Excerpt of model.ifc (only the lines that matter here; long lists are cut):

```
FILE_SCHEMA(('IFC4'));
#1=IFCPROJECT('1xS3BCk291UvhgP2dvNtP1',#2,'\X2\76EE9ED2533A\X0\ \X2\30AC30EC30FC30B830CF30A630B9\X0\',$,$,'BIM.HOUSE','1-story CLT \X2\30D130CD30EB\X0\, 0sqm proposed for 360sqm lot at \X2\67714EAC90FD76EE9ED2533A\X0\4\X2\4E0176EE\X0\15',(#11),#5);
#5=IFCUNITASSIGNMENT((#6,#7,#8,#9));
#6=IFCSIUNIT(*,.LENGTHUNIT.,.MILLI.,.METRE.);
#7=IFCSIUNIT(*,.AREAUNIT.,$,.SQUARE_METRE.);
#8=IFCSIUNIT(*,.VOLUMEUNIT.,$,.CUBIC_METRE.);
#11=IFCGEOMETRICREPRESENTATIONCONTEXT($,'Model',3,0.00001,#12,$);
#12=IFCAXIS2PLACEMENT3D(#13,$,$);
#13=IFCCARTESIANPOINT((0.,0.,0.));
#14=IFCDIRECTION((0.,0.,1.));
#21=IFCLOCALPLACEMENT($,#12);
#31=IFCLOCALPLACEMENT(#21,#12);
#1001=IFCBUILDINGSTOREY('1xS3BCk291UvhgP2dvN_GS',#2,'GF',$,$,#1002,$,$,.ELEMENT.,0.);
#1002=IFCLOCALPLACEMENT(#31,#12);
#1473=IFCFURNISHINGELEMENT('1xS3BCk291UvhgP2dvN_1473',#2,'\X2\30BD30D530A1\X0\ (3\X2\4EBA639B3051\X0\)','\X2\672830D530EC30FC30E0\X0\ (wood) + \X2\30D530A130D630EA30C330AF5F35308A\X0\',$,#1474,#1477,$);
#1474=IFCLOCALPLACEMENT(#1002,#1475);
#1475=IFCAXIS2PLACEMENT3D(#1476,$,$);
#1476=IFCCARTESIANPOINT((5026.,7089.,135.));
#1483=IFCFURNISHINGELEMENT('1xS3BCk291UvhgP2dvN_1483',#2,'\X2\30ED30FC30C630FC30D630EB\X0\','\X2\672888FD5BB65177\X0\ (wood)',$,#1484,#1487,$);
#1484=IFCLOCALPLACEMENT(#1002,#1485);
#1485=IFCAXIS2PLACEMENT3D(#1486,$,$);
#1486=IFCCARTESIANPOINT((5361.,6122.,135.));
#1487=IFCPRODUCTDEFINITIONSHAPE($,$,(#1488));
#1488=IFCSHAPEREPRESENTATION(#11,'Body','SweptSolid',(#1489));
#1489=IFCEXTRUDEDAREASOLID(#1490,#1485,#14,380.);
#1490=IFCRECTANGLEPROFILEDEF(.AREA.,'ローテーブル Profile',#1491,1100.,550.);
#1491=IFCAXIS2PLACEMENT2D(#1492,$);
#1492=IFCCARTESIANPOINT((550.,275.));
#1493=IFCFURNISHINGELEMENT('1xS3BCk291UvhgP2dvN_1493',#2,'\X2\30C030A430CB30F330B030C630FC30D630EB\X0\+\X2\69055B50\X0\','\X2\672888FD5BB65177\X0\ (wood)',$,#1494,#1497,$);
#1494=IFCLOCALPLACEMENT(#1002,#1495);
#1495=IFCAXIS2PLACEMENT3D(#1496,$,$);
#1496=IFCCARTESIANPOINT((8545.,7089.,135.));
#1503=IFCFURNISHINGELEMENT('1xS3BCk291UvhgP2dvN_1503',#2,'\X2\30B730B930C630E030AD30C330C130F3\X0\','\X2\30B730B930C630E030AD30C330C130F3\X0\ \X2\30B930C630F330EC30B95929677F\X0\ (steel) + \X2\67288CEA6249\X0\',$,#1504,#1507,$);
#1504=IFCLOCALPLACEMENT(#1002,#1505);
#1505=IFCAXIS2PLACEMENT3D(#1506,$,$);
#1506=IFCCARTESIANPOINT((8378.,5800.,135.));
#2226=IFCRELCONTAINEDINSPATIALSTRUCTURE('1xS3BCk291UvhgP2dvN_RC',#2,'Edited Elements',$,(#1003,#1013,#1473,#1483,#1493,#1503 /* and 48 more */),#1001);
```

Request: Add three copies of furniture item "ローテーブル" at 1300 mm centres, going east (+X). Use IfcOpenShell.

```python
import numpy as np
import ifcopenshell
import ifcopenshell.api.geometry
import ifcopenshell.api.root
import ifcopenshell.util.element
import ifcopenshell.util.placement
import ifcopenshell.util.unit

model = ifcopenshell.open("model.ifc")
unit_scale = ifcopenshell.util.unit.calculate_unit_scale(model)


def reuse_history(source, copy):
    """copy_class also copies each property set's owner history, people and application; keep the originals."""
    for rel in copy.IsDefinedBy:
        if rel.is_a("IfcRelDefinesByProperties") and (history := rel.RelatingPropertyDefinition.OwnerHistory):
            rel.RelatingPropertyDefinition.OwnerHistory = source.OwnerHistory
            ifcopenshell.util.element.remove_deep2(model, history)


source = model.by_guid("1xS3BCk291UvhgP2dvN_1483")
base = ifcopenshell.util.placement.get_local_placement(source.ObjectPlacement)
step = np.array([1.0, 0.0, 0.0]) * 1.3 / unit_scale

for i in range(1, 4):
    copy = ifcopenshell.api.root.copy_class(model, product=source)
    copy.Representation = ifcopenshell.util.element.copy_deep(
        model, source.Representation, exclude=["IfcGeometricRepresentationContext", "IfcRepresentationMap"]
    )
    reuse_history(source, copy)
    matrix = base.copy()
    matrix[:3, 3] += i * step
    print("added at", matrix[:3, 3].round(3) + 0.0)
    ifcopenshell.api.geometry.edit_object_placement(model, product=copy, matrix=matrix, is_si=False)

model.write("model_rev.ifc")
```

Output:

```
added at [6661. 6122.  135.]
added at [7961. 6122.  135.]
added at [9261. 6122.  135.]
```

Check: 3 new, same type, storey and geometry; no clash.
